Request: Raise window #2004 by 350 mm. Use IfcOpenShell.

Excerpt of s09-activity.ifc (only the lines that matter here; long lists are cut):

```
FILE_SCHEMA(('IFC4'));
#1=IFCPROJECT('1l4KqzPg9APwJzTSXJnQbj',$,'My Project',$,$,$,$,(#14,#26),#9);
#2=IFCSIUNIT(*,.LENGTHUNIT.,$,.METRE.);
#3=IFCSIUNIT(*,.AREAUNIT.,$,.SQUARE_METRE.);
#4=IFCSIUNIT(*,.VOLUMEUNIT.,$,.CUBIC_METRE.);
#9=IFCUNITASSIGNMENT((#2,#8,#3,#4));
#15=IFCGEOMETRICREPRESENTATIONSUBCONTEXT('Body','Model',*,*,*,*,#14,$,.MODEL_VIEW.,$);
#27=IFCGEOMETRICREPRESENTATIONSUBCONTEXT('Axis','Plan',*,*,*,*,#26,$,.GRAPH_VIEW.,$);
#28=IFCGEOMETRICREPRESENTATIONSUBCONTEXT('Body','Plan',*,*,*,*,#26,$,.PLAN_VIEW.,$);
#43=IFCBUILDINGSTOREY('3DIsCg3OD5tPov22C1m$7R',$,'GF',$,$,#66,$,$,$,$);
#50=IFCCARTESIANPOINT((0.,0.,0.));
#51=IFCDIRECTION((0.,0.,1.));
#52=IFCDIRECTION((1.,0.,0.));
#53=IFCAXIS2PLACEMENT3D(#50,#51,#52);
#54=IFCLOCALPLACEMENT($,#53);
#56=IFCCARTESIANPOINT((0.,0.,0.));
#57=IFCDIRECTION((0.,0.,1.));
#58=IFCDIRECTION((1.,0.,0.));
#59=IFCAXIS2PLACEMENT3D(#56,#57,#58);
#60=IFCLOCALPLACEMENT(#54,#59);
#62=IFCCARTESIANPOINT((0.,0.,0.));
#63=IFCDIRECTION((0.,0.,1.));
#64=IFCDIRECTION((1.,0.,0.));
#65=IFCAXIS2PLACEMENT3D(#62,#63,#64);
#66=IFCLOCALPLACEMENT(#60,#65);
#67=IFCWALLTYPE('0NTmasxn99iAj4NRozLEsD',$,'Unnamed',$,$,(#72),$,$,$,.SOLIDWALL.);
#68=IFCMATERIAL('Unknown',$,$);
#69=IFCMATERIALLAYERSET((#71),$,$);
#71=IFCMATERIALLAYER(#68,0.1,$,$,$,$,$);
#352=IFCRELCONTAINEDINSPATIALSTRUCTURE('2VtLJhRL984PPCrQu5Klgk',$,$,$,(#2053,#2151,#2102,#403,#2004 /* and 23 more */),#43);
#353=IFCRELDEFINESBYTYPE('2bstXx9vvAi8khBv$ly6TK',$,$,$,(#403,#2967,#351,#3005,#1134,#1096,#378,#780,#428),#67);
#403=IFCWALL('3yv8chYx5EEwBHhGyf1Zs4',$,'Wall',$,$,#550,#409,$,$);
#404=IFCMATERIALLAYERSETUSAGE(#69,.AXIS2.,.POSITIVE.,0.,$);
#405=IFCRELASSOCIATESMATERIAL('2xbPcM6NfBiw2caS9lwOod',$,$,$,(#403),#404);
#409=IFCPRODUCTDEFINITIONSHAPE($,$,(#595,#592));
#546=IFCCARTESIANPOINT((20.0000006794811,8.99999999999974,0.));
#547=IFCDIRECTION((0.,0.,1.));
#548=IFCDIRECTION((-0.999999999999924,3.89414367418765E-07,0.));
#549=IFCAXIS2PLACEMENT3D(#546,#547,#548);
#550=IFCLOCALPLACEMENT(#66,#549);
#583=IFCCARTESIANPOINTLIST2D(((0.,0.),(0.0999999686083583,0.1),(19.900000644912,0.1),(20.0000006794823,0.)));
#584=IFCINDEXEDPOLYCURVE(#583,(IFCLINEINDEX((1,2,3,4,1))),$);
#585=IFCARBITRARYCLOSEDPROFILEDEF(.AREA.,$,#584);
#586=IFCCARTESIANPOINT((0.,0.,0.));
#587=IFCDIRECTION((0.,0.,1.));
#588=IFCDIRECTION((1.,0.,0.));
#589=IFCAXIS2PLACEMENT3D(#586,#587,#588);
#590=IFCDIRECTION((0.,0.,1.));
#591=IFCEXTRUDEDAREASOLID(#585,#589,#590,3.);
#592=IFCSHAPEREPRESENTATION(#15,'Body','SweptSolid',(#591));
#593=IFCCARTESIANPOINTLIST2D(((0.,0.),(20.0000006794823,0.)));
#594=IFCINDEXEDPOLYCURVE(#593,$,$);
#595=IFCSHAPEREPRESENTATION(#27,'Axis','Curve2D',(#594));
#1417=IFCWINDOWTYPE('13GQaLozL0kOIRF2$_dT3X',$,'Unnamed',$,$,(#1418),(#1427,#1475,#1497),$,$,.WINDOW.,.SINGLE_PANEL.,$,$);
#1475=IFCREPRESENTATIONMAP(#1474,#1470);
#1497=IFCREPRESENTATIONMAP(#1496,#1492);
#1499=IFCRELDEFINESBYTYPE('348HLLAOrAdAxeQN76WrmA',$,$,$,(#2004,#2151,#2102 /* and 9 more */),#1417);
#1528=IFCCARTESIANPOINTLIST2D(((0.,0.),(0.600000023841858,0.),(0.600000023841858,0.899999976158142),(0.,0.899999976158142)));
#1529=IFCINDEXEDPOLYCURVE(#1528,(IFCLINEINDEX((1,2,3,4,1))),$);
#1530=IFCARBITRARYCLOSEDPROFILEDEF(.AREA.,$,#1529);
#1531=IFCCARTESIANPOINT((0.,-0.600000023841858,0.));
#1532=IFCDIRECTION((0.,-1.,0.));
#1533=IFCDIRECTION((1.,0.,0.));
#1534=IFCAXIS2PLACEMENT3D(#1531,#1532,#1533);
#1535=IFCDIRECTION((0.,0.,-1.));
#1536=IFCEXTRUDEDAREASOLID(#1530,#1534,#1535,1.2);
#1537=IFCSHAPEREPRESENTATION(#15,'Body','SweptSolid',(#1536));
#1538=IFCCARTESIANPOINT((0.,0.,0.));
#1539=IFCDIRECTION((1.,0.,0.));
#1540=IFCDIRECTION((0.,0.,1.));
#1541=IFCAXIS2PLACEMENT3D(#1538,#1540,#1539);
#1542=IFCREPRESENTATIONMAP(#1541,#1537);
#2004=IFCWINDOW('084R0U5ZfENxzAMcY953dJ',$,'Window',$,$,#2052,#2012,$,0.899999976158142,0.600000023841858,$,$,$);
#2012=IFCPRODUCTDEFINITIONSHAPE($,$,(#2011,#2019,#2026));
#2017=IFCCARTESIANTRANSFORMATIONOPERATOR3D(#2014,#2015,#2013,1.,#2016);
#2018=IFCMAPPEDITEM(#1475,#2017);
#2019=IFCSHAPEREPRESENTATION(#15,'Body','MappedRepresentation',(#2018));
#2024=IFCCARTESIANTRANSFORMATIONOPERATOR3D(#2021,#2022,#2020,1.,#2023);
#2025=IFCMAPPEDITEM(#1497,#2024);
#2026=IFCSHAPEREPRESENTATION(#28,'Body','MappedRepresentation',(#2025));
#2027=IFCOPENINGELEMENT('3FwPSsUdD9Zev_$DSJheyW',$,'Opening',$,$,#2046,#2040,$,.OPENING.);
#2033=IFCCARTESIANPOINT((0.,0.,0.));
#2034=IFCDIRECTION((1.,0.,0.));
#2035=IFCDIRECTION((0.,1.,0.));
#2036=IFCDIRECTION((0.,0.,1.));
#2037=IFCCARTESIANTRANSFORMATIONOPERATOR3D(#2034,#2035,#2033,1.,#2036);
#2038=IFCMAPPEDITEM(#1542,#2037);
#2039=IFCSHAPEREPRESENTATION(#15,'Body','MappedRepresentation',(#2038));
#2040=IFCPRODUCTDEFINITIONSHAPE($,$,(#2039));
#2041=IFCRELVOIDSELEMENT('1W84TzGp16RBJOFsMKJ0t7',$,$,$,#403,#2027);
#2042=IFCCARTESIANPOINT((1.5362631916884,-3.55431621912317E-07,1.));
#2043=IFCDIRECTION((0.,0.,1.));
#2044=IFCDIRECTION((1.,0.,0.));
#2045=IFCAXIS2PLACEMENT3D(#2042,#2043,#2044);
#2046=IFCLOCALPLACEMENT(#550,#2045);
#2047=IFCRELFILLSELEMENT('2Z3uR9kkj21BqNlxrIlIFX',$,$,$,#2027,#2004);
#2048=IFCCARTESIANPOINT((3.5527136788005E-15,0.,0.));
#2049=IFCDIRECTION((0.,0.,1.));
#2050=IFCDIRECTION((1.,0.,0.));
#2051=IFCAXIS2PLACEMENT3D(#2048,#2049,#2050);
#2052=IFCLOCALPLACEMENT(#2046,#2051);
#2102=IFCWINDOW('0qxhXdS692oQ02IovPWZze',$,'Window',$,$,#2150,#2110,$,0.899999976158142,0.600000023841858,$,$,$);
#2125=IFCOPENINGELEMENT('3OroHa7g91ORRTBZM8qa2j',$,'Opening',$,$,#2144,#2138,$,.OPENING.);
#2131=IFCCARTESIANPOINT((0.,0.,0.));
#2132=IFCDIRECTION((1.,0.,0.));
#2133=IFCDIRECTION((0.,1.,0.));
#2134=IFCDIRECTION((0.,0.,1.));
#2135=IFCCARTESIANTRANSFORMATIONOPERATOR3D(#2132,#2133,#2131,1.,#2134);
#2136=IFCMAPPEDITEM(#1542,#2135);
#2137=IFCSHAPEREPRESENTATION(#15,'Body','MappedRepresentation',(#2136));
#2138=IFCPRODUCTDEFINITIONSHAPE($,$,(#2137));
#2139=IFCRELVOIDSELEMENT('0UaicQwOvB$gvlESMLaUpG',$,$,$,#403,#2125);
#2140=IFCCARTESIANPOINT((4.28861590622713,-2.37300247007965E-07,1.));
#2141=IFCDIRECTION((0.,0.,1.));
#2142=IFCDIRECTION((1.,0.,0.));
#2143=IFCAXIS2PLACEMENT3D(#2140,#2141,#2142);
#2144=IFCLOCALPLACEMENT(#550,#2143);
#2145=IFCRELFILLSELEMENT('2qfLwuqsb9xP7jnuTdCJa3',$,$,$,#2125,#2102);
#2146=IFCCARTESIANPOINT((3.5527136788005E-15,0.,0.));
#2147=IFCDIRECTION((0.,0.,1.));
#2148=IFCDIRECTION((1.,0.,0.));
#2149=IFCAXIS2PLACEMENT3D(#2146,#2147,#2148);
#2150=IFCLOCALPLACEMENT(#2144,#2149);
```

```python
import numpy as np
import ifcopenshell
import ifcopenshell.api.geometry
import ifcopenshell.util.placement
import ifcopenshell.util.unit

model = ifcopenshell.open("s09-activity.ifc")
unit_scale = ifcopenshell.util.unit.calculate_unit_scale(model)

window = model.by_id(2004)
opening = window.FillsVoids[0].RelatingOpeningElement
dz = 0.35 / unit_scale

shift = np.array([0.0, 0.0, dz])
# The window is placed relative to its opening, so it follows when the opening moves.
matrix = ifcopenshell.util.placement.get_local_placement(opening.ObjectPlacement)
matrix[:3, 3] += shift
ifcopenshell.api.geometry.edit_object_placement(
    model, product=opening, matrix=matrix, is_si=False, should_transform_children=True
)

print(f"moved by {dz * unit_scale:+.3f} m")

model.write("s09-activity_edited.ifc")
```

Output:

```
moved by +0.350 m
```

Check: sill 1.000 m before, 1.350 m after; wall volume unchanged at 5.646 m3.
